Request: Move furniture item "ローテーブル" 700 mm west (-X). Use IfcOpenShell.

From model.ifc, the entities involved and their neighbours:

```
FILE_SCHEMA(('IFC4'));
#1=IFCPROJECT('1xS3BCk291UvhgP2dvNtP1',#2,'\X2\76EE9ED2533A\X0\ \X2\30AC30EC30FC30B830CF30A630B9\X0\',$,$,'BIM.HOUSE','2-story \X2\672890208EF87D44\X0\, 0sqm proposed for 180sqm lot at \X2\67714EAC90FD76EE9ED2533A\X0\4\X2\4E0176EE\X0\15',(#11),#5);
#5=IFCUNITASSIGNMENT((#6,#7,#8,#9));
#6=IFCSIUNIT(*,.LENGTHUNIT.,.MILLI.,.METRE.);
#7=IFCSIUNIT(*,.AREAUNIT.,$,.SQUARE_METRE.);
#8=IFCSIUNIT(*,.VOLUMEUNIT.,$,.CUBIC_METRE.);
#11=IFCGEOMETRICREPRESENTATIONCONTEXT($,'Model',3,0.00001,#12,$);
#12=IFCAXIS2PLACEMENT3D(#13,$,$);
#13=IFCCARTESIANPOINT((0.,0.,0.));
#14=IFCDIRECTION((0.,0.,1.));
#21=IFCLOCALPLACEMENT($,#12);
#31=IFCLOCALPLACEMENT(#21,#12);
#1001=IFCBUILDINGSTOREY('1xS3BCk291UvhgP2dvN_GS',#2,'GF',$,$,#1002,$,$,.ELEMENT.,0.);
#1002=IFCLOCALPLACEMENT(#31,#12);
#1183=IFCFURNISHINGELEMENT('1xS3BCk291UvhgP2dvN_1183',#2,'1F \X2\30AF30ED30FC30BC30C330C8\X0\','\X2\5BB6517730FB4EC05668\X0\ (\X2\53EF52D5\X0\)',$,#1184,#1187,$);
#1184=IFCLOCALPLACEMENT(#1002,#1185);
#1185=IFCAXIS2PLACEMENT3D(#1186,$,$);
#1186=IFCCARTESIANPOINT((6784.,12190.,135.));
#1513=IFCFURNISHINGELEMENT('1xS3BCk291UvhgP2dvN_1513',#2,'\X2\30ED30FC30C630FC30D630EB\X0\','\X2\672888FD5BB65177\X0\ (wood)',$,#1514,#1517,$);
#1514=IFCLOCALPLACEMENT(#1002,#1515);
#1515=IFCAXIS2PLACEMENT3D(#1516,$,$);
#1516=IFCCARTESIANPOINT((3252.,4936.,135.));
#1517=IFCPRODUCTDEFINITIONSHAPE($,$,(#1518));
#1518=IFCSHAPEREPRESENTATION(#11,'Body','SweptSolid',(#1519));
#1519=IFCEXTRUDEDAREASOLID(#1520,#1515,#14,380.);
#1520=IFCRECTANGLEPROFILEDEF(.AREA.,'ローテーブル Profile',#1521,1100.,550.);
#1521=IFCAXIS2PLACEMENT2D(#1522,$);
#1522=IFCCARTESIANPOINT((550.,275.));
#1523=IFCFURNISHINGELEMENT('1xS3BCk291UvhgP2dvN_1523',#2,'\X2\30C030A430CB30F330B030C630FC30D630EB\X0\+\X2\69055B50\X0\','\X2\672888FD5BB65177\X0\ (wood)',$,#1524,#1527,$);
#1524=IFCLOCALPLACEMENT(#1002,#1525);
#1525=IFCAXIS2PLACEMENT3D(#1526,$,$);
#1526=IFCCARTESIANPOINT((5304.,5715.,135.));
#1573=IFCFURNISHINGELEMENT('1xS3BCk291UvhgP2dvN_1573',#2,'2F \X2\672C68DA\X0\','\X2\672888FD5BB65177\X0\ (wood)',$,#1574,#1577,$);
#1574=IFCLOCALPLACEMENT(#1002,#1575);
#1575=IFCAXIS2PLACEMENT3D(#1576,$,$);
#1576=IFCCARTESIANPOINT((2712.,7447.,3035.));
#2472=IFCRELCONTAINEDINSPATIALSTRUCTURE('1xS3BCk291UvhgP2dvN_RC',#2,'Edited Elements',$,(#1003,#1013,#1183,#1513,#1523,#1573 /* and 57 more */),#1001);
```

```python
import ifcopenshell
import ifcopenshell.api.geometry
import ifcopenshell.util.placement
import ifcopenshell.util.unit

model = ifcopenshell.open("model.ifc")
unit_scale = ifcopenshell.util.unit.calculate_unit_scale(model)

item = model.by_id(1513)
matrix = ifcopenshell.util.placement.get_local_placement(item.ObjectPlacement)
matrix[0, 3] -= 0.7 / unit_scale
ifcopenshell.api.geometry.edit_object_placement(model, product=item, matrix=matrix, is_si=False)

print(ifcopenshell.util.placement.get_local_placement(item.ObjectPlacement).round(3) + 0.0)

model.write("model_edited.ifc")
```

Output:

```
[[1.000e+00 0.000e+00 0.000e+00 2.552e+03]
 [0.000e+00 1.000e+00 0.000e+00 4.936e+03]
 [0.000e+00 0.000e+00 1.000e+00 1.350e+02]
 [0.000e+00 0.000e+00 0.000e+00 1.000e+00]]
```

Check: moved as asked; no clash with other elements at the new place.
